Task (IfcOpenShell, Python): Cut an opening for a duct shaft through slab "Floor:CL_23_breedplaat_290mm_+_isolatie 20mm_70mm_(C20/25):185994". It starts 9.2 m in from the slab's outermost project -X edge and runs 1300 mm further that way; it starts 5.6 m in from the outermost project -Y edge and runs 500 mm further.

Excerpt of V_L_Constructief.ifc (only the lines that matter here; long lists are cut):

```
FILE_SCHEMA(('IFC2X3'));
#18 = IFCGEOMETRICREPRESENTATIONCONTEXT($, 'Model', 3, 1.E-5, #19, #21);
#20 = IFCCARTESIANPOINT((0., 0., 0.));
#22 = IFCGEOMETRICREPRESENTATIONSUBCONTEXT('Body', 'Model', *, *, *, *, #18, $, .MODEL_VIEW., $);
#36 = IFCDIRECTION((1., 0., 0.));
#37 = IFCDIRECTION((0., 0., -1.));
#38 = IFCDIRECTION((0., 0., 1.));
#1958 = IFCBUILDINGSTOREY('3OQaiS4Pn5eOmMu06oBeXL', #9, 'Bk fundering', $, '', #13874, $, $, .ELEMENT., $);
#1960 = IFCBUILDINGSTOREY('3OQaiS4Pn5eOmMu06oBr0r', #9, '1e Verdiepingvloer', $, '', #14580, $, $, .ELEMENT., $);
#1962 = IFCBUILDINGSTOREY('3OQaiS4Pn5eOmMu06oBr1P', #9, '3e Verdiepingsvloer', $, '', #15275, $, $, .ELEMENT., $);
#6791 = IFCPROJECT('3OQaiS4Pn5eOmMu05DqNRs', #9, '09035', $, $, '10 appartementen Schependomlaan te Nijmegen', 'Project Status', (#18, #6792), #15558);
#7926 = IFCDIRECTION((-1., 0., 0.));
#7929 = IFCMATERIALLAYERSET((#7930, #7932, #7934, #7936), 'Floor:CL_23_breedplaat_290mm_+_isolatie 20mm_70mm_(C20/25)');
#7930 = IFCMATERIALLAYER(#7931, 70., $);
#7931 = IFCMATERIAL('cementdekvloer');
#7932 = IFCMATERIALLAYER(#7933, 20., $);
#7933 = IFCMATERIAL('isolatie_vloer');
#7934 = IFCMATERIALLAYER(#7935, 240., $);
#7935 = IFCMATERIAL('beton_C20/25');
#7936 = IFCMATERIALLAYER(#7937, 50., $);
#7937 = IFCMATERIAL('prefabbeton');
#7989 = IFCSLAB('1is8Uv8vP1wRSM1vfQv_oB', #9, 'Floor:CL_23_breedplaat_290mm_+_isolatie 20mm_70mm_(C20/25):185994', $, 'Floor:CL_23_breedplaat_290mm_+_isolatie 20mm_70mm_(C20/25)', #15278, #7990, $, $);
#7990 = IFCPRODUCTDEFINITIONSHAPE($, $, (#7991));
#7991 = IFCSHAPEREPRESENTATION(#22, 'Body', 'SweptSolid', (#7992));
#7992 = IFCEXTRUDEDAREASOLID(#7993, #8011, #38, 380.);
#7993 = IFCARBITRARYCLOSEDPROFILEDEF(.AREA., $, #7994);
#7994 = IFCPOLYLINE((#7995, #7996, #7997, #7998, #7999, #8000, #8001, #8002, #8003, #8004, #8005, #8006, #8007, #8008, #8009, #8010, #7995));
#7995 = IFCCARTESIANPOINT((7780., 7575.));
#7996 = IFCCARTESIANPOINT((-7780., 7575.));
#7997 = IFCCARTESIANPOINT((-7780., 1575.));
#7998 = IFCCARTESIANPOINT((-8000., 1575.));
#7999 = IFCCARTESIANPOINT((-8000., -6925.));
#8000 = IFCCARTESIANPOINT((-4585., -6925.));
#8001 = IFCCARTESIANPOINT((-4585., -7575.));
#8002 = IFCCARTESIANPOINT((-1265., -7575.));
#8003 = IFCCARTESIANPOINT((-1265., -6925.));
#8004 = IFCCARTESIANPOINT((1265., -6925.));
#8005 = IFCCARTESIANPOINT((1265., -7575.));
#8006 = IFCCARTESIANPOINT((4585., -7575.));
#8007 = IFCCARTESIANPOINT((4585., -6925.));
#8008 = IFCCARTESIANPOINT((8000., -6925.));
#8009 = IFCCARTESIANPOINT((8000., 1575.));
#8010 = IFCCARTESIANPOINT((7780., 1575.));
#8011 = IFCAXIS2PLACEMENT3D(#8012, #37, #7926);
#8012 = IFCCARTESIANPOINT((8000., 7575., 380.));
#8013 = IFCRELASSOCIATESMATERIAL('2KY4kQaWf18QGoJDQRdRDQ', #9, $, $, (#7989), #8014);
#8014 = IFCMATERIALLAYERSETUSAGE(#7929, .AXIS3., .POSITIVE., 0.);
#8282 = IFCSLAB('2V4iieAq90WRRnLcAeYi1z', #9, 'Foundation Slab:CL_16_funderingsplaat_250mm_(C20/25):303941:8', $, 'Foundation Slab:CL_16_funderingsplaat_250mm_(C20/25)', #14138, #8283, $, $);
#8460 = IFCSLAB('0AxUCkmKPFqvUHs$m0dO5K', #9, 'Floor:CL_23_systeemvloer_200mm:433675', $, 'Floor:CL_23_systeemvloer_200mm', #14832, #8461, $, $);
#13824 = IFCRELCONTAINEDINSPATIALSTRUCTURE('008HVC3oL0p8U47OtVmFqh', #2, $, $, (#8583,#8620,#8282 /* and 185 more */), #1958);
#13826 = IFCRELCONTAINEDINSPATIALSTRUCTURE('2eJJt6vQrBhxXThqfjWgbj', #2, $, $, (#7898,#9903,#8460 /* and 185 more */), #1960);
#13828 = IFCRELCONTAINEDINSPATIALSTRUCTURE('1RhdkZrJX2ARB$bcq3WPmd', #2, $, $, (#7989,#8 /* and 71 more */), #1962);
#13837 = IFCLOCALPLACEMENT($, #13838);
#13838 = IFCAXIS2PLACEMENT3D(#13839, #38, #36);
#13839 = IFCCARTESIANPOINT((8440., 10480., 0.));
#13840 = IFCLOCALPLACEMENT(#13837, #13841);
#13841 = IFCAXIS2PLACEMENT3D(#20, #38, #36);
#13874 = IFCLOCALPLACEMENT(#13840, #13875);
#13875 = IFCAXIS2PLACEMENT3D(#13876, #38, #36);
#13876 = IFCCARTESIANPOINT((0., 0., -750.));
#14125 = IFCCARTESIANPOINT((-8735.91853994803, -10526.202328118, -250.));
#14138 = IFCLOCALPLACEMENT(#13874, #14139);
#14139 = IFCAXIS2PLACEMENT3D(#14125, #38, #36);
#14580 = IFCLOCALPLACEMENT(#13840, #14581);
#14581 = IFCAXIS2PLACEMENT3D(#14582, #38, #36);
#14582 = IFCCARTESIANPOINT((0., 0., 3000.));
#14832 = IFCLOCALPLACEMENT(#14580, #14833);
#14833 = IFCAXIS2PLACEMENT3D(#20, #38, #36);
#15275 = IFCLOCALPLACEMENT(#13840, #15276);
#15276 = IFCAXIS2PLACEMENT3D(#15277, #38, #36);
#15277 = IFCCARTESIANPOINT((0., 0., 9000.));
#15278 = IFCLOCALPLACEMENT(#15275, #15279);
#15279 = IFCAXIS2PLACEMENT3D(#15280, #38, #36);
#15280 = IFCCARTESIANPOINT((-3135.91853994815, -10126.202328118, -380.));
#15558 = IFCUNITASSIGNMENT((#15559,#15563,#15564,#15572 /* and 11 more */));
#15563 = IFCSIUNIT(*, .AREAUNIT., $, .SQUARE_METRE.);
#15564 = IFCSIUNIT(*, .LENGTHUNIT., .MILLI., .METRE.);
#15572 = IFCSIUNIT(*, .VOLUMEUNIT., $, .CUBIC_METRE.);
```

```python
import numpy as np
import ifcopenshell
import ifcopenshell.api.feature
import ifcopenshell.api.geometry
import ifcopenshell.api.root
import ifcopenshell.geom
import ifcopenshell.util.placement
import ifcopenshell.util.representation
import ifcopenshell.util.shape
import ifcopenshell.util.unit

model = ifcopenshell.open("V_L_Constructief.ifc")
unit_scale = ifcopenshell.util.unit.calculate_unit_scale(model)
settings = ifcopenshell.geom.settings()


def volume(element):
    """Net volume in cubic metres, openings subtracted."""
    shape = ifcopenshell.geom.create_shape(settings, element)
    return ifcopenshell.util.shape.get_volume(shape.geometry)


slab = model.by_guid("1is8Uv8vP1wRSM1vfQv_oB")
before = volume(slab)

# Extent in the slab's own axes, in metres. The edges named are its -X and -Y sides.
slab_shape = ifcopenshell.geom.create_shape(settings, slab)
vertices = ifcopenshell.util.shape.get_vertices(slab_shape.geometry)
x_min, y_min, bottom = vertices.min(axis=0)
top = vertices[:, 2].max()

opening = ifcopenshell.api.root.create_entity(model, ifc_class="IfcOpeningElement", name="Duct shaft opening")
context = ifcopenshell.util.representation.get_context(model, "Model", "Body", "MODEL_VIEW")
width, depth = 1.3, 0.5
outline = [(0.0, 0.0), (width, 0.0), (width, depth), (0.0, depth), (0.0, 0.0)]
# Overshoot both faces by 50 mm so the cut is clean.
shape = ifcopenshell.api.geometry.add_slab_representation(
    model, context=context, depth=top - bottom + 0.1, polyline=outline
)
ifcopenshell.api.geometry.assign_representation(model, product=opening, representation=shape)

matrix = ifcopenshell.util.placement.get_local_placement(slab.ObjectPlacement)
matrix[:, 3] = matrix @ np.append(np.array([x_min + 9.2, y_min + 5.6, bottom - 0.05]) / unit_scale, 1.0)
ifcopenshell.api.geometry.edit_object_placement(model, product=opening, matrix=matrix, is_si=False)
ifcopenshell.api.feature.add_feature(model, feature=opening, element=slab)

after = volume(slab)

print(f"slab volume {before:.3f} -> {after:.3f} m3")

model.write("V_L_Constructief_edited.ifc")
```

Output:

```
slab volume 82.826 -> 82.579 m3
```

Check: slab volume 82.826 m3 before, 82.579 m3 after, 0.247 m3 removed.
